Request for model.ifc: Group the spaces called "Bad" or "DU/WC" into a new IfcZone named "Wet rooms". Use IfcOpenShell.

First a look at what the model holds.

```python
import ifcopenshell

model = ifcopenshell.open("model.ifc")
print(model.schema)
seen = {}
for space in model.by_type("IfcSpace"):
    seen[space.LongName] = seen.get(space.LongName, 0) + 1
for name, count in sorted(seen.items(), key=str):
    print(count, "x", name)
print("zones:", [z.Name for z in model.by_type("IfcZone")][:20])
```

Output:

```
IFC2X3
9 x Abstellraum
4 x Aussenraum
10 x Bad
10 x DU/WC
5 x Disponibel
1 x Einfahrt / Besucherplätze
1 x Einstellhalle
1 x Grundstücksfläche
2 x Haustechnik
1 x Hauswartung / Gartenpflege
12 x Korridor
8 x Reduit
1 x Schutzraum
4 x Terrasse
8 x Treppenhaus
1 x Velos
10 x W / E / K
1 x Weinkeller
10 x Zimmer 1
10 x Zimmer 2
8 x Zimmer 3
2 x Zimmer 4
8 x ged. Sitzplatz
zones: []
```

```python
import ifcopenshell
import ifcopenshell.api.group
import ifcopenshell.api.root

model = ifcopenshell.open("model.ifc")

names = {"Bad", "DU/WC"}
spaces = [s for s in model.by_type("IfcSpace") if s.LongName in names]

zone = ifcopenshell.api.root.create_entity(model, ifc_class="IfcZone", name="Wet rooms")
ifcopenshell.api.group.assign_group(model, products=spaces, group=zone)
print(len(spaces), "spaces in", zone.Name)

model.write("model_rev.ifc")
```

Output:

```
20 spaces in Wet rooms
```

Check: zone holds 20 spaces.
